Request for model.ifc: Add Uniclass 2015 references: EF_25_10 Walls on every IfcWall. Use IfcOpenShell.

First a look at what the model holds.

```python
import ifcopenshell

model = ifcopenshell.open("model.ifc")
print(model.schema)
print("classifications:", [c.Name for c in model.by_type("IfcClassification")])
for ifc_class in ("IfcDoor", "IfcRoof", "IfcStair", "IfcWall", "IfcWindow"):
    print(ifc_class, len(model.by_type(ifc_class)))
```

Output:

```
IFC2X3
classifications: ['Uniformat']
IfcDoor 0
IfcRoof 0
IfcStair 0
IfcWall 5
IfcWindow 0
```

```python
import ifcopenshell
import ifcopenshell.api.classification

model = ifcopenshell.open("model.ifc")

# IFC2X3 requires Source and Edition and has no link from the project to the system.
system = model.create_entity("IfcClassification", Source="NBS", Edition="2015", Name="Uniclass 2015")

codes = {
    "IfcWall": ("EF_25_10", "Walls"),
}
for ifc_class, (code, name) in codes.items():
    products = model.by_type(ifc_class)
    ifcopenshell.api.classification.add_reference(
        model, products=products, classification=system, identification=code, name=name
    )
    print(code, len(products))

model.write("model-out.ifc")
```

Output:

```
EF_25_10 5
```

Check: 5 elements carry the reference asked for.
